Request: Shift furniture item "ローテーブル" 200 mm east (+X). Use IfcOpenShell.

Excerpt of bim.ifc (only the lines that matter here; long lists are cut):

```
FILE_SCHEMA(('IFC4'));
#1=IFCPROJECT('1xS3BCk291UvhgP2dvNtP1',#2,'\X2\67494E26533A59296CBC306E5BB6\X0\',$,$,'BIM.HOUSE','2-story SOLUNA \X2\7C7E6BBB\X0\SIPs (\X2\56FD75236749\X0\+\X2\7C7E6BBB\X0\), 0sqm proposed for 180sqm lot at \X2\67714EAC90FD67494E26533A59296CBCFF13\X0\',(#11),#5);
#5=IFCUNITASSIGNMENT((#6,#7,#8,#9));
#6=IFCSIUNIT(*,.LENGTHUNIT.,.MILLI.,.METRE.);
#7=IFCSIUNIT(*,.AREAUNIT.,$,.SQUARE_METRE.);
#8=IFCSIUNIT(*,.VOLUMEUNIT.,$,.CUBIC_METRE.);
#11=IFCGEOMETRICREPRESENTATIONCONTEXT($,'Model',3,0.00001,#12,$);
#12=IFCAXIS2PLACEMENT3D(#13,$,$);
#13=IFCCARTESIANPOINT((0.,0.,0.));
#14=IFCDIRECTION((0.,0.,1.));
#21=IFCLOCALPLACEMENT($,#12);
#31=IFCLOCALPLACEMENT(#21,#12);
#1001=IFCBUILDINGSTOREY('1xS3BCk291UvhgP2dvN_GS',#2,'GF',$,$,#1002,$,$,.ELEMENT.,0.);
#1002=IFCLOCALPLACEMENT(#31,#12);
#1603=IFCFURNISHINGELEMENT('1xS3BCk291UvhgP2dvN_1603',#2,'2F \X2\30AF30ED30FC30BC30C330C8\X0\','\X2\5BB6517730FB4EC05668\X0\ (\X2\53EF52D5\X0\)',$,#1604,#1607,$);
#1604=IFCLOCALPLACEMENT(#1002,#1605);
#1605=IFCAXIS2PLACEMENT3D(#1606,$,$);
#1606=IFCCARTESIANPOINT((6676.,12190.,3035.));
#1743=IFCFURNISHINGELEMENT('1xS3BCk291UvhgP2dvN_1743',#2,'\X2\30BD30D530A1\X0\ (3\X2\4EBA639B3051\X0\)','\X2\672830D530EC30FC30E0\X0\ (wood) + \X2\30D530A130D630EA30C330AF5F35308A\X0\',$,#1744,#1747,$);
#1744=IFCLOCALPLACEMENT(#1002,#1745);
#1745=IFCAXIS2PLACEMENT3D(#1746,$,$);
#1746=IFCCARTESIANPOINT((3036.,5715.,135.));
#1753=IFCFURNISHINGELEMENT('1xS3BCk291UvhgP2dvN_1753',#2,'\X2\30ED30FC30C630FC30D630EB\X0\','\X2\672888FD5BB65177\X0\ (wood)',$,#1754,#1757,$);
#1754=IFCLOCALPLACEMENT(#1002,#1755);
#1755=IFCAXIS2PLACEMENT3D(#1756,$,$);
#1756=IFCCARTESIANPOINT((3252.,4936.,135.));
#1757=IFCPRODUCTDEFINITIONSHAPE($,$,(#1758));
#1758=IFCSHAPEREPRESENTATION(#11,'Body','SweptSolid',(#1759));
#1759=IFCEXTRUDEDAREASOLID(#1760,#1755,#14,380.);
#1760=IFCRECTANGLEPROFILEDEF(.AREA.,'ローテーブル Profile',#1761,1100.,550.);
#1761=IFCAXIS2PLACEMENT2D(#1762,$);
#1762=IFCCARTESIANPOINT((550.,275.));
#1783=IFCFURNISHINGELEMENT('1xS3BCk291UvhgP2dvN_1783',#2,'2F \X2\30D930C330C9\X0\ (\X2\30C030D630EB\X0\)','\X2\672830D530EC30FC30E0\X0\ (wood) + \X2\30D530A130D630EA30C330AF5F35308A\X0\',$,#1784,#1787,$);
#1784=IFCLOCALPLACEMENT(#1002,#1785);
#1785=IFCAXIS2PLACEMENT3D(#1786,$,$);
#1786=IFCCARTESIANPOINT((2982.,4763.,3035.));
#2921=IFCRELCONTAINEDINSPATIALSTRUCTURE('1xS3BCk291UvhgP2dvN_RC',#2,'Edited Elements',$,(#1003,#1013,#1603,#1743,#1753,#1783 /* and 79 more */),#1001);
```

```python
import ifcopenshell
import ifcopenshell.api.geometry
import ifcopenshell.util.placement
import ifcopenshell.util.unit

model = ifcopenshell.open("bim.ifc")
unit_scale = ifcopenshell.util.unit.calculate_unit_scale(model)

item = model.by_guid("1xS3BCk291UvhgP2dvN_1753")
matrix = ifcopenshell.util.placement.get_local_placement(item.ObjectPlacement)
matrix[0, 3] += 0.2 / unit_scale
ifcopenshell.api.geometry.edit_object_placement(model, product=item, matrix=matrix, is_si=False)

print(ifcopenshell.util.placement.get_local_placement(item.ObjectPlacement).round(3) + 0.0)

model.write("bim_edited.ifc")
```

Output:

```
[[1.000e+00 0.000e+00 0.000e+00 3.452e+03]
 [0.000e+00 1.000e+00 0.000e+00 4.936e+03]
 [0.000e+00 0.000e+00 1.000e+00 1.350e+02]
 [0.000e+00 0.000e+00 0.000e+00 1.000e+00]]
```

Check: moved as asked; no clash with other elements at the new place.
